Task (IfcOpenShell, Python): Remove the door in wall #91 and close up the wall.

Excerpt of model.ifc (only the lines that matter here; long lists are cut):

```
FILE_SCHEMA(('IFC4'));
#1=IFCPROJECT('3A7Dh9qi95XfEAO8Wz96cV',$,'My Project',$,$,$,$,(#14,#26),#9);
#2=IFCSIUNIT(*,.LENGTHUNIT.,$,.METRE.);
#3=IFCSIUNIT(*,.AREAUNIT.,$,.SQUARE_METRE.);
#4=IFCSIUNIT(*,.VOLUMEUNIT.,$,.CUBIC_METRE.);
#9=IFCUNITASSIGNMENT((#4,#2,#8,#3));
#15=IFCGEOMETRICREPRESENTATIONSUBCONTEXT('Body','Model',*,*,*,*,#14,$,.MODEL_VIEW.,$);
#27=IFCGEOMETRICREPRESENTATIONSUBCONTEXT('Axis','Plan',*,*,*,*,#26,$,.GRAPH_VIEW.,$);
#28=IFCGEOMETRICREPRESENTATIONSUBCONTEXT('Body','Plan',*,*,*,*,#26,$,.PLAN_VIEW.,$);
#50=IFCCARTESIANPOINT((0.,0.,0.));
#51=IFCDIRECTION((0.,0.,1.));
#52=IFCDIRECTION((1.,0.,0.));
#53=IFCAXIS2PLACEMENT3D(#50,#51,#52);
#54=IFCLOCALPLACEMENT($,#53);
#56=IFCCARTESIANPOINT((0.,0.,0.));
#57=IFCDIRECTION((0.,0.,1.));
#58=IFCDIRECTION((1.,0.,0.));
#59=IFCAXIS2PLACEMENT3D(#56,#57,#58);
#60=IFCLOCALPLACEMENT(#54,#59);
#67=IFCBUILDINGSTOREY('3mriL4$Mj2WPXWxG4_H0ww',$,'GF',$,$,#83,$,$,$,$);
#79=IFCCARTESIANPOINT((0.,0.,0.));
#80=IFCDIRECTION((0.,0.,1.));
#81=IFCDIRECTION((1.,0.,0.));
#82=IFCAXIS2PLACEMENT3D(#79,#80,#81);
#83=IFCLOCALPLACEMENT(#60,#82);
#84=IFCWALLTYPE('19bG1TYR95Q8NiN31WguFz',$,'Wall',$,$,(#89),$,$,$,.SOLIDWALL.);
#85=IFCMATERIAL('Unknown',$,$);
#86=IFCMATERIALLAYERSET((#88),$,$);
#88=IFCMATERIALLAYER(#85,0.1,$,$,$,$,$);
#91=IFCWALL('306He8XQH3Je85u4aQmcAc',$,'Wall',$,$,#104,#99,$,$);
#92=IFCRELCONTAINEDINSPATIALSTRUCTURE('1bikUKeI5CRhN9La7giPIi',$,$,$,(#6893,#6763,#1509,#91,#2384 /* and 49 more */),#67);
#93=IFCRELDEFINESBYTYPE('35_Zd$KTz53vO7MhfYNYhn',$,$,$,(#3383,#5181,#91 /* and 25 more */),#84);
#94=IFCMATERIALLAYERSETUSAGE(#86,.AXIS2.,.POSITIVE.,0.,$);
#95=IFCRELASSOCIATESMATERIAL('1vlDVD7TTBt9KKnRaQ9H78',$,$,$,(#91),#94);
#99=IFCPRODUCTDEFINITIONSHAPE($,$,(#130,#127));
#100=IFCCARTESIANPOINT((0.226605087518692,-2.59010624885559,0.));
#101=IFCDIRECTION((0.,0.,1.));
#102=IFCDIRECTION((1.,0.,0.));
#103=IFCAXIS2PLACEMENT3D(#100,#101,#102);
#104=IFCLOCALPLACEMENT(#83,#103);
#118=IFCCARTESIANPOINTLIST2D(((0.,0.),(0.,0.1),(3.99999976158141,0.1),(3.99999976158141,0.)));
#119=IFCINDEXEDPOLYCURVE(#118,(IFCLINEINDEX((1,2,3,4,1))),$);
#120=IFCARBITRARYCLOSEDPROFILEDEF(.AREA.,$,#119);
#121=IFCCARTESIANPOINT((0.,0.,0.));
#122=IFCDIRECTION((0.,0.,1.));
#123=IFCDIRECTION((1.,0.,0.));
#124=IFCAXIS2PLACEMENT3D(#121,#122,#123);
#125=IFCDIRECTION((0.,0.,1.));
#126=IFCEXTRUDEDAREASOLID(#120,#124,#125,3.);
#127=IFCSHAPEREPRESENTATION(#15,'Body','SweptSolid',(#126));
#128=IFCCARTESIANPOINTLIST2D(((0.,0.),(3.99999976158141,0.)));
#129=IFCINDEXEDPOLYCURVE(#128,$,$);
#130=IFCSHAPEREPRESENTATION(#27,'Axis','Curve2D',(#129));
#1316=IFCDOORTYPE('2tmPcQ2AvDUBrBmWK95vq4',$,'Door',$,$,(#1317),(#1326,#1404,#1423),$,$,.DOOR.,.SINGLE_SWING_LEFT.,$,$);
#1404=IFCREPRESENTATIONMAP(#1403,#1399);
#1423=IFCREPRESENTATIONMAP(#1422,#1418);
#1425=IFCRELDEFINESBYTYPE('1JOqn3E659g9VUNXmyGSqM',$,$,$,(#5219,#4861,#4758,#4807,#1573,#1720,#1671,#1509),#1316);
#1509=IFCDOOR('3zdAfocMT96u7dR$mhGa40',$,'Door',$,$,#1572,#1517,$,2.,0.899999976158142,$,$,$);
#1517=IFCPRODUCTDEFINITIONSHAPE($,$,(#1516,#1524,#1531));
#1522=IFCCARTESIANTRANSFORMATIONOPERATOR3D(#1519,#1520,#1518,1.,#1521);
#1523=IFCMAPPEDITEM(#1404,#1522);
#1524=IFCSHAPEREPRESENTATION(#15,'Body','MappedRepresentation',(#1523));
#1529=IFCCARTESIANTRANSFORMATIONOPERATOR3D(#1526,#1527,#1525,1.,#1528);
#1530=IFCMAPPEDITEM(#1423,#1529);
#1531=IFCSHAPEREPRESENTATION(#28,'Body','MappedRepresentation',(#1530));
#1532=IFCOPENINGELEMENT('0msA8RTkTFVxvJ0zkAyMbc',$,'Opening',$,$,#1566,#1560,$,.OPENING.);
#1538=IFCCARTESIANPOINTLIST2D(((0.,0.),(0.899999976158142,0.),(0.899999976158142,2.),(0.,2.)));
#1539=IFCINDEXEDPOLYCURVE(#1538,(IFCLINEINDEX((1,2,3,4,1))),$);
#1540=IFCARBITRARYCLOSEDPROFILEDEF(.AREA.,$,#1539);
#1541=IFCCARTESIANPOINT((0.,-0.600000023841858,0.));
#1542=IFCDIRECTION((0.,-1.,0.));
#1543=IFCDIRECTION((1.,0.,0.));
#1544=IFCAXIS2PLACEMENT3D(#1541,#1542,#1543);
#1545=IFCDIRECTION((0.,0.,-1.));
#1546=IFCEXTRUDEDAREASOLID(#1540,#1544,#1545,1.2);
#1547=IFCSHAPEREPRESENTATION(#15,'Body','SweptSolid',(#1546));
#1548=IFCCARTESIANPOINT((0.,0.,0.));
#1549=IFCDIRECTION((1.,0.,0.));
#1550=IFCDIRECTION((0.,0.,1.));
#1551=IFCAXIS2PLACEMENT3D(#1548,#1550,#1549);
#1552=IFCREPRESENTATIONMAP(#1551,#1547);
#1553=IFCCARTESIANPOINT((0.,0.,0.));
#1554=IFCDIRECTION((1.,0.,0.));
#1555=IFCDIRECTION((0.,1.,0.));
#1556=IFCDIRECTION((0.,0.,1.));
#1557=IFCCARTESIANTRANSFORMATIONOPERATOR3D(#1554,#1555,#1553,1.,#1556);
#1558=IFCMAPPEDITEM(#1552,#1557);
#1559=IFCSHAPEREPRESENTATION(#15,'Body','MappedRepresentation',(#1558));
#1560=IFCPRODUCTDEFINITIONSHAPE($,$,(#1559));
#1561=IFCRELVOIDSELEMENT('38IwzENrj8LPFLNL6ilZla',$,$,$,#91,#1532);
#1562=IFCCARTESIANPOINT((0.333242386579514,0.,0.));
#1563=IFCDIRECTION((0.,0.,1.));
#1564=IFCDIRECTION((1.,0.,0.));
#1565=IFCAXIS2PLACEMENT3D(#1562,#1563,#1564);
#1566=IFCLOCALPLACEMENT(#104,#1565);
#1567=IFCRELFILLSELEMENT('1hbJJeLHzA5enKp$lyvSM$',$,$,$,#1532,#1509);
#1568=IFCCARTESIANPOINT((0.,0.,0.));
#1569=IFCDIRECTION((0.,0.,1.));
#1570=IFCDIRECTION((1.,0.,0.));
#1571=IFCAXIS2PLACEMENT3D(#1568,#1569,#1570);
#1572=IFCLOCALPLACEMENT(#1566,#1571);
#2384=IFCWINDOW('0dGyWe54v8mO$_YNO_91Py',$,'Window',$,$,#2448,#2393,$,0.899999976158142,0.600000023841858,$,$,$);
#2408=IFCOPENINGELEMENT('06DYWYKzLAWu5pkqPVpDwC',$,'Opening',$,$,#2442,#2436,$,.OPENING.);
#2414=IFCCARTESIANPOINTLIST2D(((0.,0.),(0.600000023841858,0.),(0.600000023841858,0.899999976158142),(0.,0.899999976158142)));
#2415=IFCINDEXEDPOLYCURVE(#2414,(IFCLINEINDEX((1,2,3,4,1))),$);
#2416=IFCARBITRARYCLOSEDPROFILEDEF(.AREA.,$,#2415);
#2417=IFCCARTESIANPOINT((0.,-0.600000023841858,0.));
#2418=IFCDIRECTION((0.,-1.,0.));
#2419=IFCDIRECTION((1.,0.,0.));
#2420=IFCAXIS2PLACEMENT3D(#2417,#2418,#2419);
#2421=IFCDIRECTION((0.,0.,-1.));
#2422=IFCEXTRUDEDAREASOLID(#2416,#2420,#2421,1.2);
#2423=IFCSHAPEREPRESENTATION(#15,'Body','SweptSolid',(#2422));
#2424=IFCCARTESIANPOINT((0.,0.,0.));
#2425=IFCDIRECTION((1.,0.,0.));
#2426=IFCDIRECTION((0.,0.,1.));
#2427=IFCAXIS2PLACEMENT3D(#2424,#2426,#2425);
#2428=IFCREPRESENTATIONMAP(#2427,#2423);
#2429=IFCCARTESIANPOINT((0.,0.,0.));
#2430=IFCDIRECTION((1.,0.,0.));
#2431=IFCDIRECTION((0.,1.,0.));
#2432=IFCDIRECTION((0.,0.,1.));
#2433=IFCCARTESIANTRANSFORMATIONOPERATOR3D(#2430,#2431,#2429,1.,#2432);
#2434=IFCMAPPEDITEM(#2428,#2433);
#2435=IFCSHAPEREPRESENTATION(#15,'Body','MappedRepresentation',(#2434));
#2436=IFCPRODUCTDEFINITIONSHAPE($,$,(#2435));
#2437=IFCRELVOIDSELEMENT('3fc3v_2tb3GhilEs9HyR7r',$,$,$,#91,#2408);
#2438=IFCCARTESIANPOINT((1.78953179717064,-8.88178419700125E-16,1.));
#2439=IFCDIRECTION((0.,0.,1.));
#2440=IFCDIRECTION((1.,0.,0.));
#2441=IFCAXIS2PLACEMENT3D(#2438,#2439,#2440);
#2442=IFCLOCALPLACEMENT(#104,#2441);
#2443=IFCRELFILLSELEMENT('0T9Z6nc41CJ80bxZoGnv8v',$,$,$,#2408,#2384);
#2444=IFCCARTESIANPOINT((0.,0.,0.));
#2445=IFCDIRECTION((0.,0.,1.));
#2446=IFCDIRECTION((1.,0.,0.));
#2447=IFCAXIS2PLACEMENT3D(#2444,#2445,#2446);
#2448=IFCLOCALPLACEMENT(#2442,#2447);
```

```python
import ifcopenshell
import ifcopenshell.api.feature
import ifcopenshell.api.root
import ifcopenshell.geom
import ifcopenshell.util.shape

model = ifcopenshell.open("model.ifc")
settings = ifcopenshell.geom.settings()


def volume(element):
    """Net volume in cubic metres, openings subtracted."""
    shape = ifcopenshell.geom.create_shape(settings, element)
    return ifcopenshell.util.shape.get_volume(shape.geometry)


door = model.by_id(1509)
opening = door.FillsVoids[0].RelatingOpeningElement
wall = opening.VoidsElements[0].RelatingBuildingElement
before = volume(wall)

ifcopenshell.api.root.remove_product(model, product=door)
ifcopenshell.api.feature.remove_feature(model, feature=opening)

after = volume(wall)

print(f"wall volume {before:.3f} -> {after:.3f} m3")

model.write("model_updated.ifc")
```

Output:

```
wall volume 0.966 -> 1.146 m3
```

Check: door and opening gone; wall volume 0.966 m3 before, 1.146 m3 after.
